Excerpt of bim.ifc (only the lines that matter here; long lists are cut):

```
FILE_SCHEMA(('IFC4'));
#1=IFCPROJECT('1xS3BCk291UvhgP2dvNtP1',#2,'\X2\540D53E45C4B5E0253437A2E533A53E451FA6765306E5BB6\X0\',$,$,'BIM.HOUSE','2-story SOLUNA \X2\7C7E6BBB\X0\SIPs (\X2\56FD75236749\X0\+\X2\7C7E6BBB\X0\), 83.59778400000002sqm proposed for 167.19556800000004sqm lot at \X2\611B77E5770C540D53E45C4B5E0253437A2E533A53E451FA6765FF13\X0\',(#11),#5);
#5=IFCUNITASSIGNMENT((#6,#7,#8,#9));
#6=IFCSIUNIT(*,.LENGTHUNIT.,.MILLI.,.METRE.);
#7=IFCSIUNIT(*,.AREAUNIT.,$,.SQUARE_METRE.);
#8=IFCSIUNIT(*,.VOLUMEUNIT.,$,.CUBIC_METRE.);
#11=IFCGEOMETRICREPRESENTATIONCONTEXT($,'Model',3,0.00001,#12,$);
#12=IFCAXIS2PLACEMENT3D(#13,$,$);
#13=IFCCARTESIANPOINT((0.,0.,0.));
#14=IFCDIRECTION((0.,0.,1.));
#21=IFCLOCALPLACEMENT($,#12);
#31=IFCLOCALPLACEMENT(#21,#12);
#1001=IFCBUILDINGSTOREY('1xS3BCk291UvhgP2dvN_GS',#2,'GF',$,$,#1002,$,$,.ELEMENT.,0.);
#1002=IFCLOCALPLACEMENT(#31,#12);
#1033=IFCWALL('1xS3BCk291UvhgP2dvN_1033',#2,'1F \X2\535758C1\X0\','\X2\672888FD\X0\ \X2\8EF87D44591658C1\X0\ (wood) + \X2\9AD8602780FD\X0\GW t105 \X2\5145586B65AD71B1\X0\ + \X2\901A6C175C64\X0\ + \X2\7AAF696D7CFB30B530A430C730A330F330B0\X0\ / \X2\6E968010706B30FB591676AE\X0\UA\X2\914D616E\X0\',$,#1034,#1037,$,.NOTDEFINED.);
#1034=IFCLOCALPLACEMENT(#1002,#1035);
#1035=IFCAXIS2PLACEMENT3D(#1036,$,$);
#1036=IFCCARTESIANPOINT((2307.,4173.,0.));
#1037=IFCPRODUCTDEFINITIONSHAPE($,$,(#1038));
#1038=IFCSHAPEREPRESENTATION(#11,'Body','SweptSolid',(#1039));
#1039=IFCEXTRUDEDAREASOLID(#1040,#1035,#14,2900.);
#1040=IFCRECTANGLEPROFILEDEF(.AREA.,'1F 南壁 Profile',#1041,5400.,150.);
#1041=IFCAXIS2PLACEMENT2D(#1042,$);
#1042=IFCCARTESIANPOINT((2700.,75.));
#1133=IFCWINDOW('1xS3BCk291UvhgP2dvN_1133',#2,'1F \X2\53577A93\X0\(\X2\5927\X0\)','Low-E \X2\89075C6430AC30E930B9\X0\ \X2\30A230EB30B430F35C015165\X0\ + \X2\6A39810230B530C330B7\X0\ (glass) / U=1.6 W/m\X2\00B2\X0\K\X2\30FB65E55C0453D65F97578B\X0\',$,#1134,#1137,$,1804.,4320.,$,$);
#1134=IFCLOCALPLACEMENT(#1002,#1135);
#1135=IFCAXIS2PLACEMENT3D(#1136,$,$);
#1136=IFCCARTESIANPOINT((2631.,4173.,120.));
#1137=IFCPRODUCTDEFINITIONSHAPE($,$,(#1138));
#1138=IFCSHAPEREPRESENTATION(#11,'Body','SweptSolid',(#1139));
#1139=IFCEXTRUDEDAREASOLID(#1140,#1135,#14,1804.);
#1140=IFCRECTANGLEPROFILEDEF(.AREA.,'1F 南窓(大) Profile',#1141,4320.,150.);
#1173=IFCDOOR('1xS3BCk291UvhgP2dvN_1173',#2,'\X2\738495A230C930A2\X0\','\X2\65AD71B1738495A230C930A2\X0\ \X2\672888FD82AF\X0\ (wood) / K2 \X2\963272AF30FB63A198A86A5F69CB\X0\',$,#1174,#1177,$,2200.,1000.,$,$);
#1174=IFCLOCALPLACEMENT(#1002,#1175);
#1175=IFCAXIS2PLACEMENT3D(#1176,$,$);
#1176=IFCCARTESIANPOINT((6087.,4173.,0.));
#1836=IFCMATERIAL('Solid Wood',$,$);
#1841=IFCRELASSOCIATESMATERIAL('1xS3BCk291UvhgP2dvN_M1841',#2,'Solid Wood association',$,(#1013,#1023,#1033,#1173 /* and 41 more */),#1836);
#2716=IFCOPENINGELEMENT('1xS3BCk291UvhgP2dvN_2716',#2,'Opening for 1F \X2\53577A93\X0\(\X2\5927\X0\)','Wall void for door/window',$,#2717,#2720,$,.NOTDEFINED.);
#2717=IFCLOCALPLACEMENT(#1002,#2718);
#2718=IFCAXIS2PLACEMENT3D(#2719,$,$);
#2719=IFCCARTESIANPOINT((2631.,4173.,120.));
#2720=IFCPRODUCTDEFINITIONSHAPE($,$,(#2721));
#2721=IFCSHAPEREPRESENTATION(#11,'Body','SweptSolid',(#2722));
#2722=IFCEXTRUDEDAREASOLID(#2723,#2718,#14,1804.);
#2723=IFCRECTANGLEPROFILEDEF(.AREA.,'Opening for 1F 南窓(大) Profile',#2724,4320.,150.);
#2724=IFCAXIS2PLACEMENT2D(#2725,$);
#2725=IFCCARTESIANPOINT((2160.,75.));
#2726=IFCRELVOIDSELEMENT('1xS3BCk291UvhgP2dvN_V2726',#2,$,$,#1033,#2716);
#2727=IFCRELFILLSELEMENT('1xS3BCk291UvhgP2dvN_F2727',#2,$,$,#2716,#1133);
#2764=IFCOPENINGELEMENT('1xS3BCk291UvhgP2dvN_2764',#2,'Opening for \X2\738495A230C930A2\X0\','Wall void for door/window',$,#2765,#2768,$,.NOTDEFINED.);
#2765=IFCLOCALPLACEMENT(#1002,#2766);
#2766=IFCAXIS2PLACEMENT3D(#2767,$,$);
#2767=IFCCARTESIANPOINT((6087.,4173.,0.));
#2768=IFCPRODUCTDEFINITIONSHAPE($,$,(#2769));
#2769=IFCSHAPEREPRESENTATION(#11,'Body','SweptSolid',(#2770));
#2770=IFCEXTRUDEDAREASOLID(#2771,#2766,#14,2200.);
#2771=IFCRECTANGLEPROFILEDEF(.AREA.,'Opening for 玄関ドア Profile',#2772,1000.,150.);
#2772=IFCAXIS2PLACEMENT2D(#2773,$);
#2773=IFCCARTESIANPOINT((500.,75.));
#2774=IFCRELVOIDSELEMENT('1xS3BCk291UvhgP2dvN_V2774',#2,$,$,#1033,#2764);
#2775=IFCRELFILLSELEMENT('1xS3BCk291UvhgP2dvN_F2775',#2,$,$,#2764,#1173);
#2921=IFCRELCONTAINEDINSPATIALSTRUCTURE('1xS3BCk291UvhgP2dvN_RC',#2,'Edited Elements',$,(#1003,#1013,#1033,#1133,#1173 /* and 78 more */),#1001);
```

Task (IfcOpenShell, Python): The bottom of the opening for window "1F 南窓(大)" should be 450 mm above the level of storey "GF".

```python
import numpy as np
import ifcopenshell
import ifcopenshell.api.geometry
import ifcopenshell.geom
import ifcopenshell.util.element
import ifcopenshell.util.placement
import ifcopenshell.util.shape
import ifcopenshell.util.unit

model = ifcopenshell.open("bim.ifc")
unit_scale = ifcopenshell.util.unit.calculate_unit_scale(model)

window = model.by_guid("1xS3BCk291UvhgP2dvN_1133")
opening = window.FillsVoids[0].RelatingOpeningElement
storey = ifcopenshell.util.element.get_container(window, ifc_class="IfcBuildingStorey")
level = ifcopenshell.util.placement.get_local_placement(storey.ObjectPlacement)[2, 3]

# The opening's origin need not be at the sill, so measure its lowest point.
shape = ifcopenshell.geom.create_shape(ifcopenshell.geom.settings(), opening)
bottom = ifcopenshell.util.shape.get_shape_bottom_elevation(shape, shape.geometry) / unit_scale
dz = level + 450.0 - bottom

shift = np.array([0.0, 0.0, dz])
# The window is not placed relative to its opening, so move both.
for product in (opening, window):
    matrix = ifcopenshell.util.placement.get_local_placement(product.ObjectPlacement)
    matrix[:3, 3] += shift
    ifcopenshell.api.geometry.edit_object_placement(model, product=product, matrix=matrix, is_si=False)

print(f"moved by {dz * unit_scale:+.3f} m")

model.write("bim_updated.ifc")
```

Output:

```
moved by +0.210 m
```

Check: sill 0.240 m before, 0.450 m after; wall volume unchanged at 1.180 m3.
